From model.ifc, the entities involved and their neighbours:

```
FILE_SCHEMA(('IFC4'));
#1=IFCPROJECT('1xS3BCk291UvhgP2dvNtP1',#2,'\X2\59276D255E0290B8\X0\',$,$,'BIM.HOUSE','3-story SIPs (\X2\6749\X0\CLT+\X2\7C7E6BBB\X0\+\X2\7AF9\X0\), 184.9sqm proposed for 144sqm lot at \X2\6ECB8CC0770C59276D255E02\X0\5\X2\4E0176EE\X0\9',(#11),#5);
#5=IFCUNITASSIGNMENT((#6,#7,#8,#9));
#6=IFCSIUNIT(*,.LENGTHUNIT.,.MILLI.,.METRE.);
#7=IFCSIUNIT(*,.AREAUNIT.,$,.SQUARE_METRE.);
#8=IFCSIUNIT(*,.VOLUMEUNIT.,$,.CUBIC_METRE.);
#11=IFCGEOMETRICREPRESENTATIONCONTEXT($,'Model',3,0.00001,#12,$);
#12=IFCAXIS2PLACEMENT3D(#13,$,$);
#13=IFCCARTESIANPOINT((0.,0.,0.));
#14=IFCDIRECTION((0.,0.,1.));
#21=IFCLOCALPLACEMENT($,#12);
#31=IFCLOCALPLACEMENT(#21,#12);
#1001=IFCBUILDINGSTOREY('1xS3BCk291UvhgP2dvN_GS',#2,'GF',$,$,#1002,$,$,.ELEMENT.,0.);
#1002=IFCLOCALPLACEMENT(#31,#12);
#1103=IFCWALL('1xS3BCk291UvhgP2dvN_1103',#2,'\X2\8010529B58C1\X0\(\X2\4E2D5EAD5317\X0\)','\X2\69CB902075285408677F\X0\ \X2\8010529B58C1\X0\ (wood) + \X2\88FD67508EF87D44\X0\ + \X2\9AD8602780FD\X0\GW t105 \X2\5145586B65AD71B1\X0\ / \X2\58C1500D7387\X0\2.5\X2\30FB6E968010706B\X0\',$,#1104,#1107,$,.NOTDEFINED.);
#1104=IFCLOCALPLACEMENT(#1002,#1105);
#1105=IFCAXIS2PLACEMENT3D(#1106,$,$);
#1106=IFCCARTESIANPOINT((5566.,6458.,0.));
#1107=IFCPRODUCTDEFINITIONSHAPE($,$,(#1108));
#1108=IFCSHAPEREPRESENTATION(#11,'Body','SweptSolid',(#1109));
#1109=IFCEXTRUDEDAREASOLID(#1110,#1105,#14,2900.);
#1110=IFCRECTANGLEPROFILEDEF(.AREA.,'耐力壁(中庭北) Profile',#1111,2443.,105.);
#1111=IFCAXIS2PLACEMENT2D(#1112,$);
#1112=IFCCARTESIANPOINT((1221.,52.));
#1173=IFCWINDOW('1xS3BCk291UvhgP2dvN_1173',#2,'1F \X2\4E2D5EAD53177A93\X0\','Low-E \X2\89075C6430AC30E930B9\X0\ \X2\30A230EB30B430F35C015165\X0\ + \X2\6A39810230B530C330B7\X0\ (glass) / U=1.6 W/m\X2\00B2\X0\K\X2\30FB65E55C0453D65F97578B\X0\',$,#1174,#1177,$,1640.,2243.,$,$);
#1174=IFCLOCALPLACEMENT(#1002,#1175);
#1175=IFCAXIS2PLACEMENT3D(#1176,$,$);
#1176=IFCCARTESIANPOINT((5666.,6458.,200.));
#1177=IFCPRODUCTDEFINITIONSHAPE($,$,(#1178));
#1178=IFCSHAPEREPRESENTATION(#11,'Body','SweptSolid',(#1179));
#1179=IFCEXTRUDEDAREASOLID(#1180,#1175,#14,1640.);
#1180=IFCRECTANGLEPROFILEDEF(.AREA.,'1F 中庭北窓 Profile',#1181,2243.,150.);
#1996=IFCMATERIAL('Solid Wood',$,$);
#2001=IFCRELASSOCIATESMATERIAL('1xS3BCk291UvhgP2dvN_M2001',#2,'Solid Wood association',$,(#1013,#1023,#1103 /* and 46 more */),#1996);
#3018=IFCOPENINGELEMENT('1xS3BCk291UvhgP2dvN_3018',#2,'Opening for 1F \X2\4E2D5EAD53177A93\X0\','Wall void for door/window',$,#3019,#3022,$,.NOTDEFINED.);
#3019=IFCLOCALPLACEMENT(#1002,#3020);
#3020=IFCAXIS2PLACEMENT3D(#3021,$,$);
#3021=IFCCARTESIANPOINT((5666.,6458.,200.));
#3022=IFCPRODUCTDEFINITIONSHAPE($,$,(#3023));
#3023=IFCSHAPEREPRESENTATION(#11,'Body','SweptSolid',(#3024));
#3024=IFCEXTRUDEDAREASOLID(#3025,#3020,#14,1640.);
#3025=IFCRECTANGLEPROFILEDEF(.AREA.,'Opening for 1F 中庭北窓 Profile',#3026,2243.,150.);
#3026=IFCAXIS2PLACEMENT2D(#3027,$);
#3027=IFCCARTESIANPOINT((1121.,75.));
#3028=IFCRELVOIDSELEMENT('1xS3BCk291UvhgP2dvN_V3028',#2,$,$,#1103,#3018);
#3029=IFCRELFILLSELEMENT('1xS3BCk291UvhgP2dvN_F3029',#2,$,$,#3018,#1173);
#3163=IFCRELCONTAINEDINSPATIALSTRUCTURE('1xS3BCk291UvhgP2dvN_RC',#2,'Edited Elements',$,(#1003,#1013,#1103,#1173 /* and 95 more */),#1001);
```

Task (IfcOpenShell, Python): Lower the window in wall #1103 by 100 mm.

```python
import numpy as np
import ifcopenshell
import ifcopenshell.api.geometry
import ifcopenshell.util.placement
import ifcopenshell.util.unit

model = ifcopenshell.open("model.ifc")
unit_scale = ifcopenshell.util.unit.calculate_unit_scale(model)

window = model.by_guid("1xS3BCk291UvhgP2dvN_1173")
opening = window.FillsVoids[0].RelatingOpeningElement
dz = -0.1 / unit_scale

shift = np.array([0.0, 0.0, dz])
# The window is not placed relative to its opening, so move both.
for product in (opening, window):
    matrix = ifcopenshell.util.placement.get_local_placement(product.ObjectPlacement)
    matrix[:3, 3] += shift
    ifcopenshell.api.geometry.edit_object_placement(model, product=product, matrix=matrix, is_si=False)

print(f"moved by {dz * unit_scale:+.3f} m")

model.write("model-out.ifc")
```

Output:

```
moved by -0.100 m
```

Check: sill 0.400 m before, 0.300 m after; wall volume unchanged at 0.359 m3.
